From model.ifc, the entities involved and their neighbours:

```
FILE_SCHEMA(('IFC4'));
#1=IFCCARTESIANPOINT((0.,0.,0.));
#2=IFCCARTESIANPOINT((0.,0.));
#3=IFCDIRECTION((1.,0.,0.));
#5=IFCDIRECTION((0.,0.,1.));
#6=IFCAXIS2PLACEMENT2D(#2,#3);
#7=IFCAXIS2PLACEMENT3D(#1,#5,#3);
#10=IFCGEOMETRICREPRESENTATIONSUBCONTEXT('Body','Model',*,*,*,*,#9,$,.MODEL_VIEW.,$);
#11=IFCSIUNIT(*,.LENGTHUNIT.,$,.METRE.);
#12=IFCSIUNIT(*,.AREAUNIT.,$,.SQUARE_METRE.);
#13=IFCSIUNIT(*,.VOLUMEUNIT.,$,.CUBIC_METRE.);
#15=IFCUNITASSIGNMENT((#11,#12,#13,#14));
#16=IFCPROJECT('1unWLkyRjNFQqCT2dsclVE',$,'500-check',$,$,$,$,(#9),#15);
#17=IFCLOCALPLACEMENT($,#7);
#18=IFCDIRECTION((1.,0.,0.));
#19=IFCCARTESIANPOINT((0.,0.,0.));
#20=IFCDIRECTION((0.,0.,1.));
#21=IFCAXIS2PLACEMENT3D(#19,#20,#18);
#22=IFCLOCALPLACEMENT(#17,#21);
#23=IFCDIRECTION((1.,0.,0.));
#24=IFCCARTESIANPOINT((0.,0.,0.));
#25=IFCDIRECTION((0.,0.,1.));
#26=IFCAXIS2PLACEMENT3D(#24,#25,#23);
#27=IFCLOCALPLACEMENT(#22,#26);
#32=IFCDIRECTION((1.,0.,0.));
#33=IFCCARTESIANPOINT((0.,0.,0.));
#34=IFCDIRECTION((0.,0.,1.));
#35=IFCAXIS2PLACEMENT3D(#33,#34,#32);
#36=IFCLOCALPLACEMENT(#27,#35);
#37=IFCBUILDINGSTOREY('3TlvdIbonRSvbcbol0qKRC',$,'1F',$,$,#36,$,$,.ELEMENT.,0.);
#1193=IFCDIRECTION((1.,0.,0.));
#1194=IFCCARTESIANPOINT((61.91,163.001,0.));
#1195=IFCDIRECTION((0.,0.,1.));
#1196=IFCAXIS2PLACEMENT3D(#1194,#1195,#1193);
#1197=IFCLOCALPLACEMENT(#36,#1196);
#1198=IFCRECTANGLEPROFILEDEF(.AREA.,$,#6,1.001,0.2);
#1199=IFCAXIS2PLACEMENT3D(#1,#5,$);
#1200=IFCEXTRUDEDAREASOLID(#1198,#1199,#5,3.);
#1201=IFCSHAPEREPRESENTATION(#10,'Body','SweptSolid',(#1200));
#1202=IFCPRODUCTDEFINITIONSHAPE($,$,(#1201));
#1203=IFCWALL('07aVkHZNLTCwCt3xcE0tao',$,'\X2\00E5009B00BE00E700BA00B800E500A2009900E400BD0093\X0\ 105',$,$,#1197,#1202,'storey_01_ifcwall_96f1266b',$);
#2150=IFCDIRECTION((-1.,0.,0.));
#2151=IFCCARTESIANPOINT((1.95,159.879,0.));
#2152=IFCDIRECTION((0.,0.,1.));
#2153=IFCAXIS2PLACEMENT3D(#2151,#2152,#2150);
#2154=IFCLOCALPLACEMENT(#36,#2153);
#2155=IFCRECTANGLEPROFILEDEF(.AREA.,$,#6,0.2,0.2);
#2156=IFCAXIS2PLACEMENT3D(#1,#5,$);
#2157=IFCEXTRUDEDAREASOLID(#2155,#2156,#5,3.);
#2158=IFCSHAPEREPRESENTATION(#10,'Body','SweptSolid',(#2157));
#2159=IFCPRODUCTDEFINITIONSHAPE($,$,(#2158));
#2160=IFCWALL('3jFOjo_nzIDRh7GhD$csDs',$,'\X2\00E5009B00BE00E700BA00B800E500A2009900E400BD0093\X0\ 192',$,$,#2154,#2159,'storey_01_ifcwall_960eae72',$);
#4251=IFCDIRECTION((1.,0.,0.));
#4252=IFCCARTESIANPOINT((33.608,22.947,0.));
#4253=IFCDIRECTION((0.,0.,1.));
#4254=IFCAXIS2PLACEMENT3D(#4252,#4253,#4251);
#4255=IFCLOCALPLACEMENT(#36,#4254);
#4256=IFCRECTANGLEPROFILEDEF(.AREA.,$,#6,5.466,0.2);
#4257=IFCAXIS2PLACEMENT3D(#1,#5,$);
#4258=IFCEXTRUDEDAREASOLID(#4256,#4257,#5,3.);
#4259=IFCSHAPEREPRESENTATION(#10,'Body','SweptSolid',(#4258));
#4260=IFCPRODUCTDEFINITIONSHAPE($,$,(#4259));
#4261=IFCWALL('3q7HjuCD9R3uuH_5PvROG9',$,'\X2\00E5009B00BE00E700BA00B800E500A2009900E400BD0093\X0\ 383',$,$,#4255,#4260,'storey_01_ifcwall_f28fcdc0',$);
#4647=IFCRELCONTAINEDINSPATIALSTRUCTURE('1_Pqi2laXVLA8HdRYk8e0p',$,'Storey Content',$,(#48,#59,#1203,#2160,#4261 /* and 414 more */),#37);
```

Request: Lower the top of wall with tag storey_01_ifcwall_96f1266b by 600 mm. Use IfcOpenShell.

```python
import ifcopenshell
import ifcopenshell.geom
import ifcopenshell.util.representation
import ifcopenshell.util.shape

model = ifcopenshell.open("model.ifc")
settings = ifcopenshell.geom.settings()


def volume(element):
    """Net volume in cubic metres, openings subtracted."""
    shape = ifcopenshell.geom.create_shape(settings, element)
    return ifcopenshell.util.shape.get_volume(shape.geometry)


wall = model.by_id(1203)
before = volume(wall)

body = ifcopenshell.util.representation.get_representation(wall, "Model", "Body")
solid = body.Items[0]
old_height = solid.Depth
solid.Depth -= 0.6
after = volume(wall)

print(f"height {old_height:g} -> {solid.Depth:g}, volume {before:.3f} -> {after:.3f} m3")

model.write("model-out.ifc")
```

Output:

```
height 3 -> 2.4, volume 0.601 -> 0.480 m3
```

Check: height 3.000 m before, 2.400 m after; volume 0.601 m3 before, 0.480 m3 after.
